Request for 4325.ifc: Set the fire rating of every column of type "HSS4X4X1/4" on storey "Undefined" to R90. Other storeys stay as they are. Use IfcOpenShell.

First a look at what the model holds.

```python
import ifcopenshell
import ifcopenshell.util.element

model = ifcopenshell.open("4325.ifc")
print(model.schema)
storey = next(s for s in model.by_type("IfcBuildingStorey") if s.Name == "Undefined")
columns = [e for e in ifcopenshell.util.element.get_decomposition(storey) if e.is_a("IfcColumn")]
seen = {}
for e in columns:
    element_type = ifcopenshell.util.element.get_type(e)
    key = (element_type.Name if element_type != e and element_type else None, ifcopenshell.util.element.get_pset(e, "Pset_ColumnCommon", "FireRating"))
    seen[key] = seen.get(key, 0) + 1
for (name, value), count in sorted(seen.items(), key=str):
    print(count, "x", name, "|", value)
```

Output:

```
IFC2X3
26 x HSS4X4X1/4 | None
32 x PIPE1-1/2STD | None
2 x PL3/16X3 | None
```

```python
import ifcopenshell
import ifcopenshell.api.pset
import ifcopenshell.util.element

model = ifcopenshell.open("4325.ifc")

storey = next(s for s in model.by_type("IfcBuildingStorey") if s.Name == "Undefined")
columns = [e for e in ifcopenshell.util.element.get_decomposition(storey) if e.is_a("IfcColumn")]

count = 0
for e in columns:
    element_type = ifcopenshell.util.element.get_type(e)
    if element_type in (None, e) or element_type.Name != "HSS4X4X1/4":
        continue
    found = ifcopenshell.util.element.get_pset(e, "Pset_ColumnCommon", should_inherit=False)
    if found:
        pset = model.by_id(found["id"])
        if len(ifcopenshell.util.element.get_elements_by_pset(pset)) > 1:
            pset = ifcopenshell.api.pset.unshare_pset(model, products=[e], pset=pset)[0]
    else:
        pset = ifcopenshell.api.pset.add_pset(model, product=e, name="Pset_ColumnCommon")
    ifcopenshell.api.pset.edit_pset(model, pset=pset, properties={"FireRating": "R90"})
    count += 1

print(count, "columns updated")

model.write("4325_edited.ifc")
```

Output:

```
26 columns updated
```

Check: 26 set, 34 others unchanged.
